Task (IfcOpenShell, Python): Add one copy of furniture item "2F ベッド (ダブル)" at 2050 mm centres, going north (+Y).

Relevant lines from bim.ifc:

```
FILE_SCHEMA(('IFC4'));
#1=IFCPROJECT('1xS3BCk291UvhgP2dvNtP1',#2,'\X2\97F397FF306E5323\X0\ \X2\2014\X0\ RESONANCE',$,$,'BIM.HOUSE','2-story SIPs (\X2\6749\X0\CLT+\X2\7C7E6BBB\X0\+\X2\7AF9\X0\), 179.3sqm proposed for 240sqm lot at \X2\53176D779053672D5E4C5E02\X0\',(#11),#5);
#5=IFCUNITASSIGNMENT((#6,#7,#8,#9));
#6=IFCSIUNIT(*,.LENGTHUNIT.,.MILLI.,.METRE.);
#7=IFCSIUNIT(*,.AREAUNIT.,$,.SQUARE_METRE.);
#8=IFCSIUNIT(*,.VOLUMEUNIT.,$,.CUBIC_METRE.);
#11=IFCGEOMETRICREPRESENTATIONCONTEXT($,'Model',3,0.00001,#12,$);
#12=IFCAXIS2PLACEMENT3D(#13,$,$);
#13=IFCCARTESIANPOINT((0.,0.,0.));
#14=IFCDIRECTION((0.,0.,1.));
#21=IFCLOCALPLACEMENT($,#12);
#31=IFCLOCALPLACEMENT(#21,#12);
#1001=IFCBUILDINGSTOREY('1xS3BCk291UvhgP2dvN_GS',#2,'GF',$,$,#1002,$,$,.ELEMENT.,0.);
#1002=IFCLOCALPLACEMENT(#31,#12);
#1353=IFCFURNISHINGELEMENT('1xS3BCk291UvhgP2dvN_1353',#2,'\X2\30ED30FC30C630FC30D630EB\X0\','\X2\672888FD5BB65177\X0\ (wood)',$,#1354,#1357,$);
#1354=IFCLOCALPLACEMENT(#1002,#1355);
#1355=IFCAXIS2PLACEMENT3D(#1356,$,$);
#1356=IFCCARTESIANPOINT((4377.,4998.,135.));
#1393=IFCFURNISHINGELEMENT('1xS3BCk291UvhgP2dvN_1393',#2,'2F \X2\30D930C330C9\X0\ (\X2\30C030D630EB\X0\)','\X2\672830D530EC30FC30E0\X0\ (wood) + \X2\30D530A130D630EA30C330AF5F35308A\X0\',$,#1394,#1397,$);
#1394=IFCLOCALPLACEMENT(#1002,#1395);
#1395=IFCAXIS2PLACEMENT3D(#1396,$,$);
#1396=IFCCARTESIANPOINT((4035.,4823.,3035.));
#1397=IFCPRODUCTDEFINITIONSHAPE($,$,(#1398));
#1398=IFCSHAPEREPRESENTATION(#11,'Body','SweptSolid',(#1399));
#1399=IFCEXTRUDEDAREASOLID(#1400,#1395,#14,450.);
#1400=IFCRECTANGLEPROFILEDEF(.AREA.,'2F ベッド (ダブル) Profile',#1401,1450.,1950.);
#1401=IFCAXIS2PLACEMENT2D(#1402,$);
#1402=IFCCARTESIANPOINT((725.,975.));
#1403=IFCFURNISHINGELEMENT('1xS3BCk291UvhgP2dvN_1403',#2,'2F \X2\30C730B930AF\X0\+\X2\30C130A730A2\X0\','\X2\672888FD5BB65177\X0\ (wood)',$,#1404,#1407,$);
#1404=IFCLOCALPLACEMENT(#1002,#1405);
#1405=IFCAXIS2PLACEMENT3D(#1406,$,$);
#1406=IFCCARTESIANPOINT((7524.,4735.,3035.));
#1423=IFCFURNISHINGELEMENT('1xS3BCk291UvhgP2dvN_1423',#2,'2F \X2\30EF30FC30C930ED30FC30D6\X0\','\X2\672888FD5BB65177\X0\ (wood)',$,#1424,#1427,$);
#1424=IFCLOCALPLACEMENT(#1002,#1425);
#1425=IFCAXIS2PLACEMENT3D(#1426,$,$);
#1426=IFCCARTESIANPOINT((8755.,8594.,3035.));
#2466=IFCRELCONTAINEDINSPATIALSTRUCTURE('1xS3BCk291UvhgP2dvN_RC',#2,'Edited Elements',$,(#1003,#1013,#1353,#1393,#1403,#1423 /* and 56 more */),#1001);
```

```python
import numpy as np
import ifcopenshell
import ifcopenshell.api.geometry
import ifcopenshell.api.root
import ifcopenshell.util.element
import ifcopenshell.util.placement
import ifcopenshell.util.unit

model = ifcopenshell.open("bim.ifc")
unit_scale = ifcopenshell.util.unit.calculate_unit_scale(model)


def reuse_history(source, copy):
    """copy_class also copies each property set's owner history, people and application; keep the originals."""
    for rel in copy.IsDefinedBy:
        if rel.is_a("IfcRelDefinesByProperties") and (history := rel.RelatingPropertyDefinition.OwnerHistory):
            rel.RelatingPropertyDefinition.OwnerHistory = source.OwnerHistory
            ifcopenshell.util.element.remove_deep2(model, history)


source = model.by_guid("1xS3BCk291UvhgP2dvN_1393")
base = ifcopenshell.util.placement.get_local_placement(source.ObjectPlacement)
step = np.array([0.0, 1.0, 0.0]) * 2.05 / unit_scale

for i in range(1, 2):
    copy = ifcopenshell.api.root.copy_class(model, product=source)
    copy.Representation = ifcopenshell.util.element.copy_deep(
        model, source.Representation, exclude=["IfcGeometricRepresentationContext", "IfcRepresentationMap"]
    )
    reuse_history(source, copy)
    matrix = base.copy()
    matrix[:3, 3] += i * step
    print("added at", matrix[:3, 3].round(3) + 0.0)
    ifcopenshell.api.geometry.edit_object_placement(model, product=copy, matrix=matrix, is_si=False)

model.write("bim-out.ifc")
```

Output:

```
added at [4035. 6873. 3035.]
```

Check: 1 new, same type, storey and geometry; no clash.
